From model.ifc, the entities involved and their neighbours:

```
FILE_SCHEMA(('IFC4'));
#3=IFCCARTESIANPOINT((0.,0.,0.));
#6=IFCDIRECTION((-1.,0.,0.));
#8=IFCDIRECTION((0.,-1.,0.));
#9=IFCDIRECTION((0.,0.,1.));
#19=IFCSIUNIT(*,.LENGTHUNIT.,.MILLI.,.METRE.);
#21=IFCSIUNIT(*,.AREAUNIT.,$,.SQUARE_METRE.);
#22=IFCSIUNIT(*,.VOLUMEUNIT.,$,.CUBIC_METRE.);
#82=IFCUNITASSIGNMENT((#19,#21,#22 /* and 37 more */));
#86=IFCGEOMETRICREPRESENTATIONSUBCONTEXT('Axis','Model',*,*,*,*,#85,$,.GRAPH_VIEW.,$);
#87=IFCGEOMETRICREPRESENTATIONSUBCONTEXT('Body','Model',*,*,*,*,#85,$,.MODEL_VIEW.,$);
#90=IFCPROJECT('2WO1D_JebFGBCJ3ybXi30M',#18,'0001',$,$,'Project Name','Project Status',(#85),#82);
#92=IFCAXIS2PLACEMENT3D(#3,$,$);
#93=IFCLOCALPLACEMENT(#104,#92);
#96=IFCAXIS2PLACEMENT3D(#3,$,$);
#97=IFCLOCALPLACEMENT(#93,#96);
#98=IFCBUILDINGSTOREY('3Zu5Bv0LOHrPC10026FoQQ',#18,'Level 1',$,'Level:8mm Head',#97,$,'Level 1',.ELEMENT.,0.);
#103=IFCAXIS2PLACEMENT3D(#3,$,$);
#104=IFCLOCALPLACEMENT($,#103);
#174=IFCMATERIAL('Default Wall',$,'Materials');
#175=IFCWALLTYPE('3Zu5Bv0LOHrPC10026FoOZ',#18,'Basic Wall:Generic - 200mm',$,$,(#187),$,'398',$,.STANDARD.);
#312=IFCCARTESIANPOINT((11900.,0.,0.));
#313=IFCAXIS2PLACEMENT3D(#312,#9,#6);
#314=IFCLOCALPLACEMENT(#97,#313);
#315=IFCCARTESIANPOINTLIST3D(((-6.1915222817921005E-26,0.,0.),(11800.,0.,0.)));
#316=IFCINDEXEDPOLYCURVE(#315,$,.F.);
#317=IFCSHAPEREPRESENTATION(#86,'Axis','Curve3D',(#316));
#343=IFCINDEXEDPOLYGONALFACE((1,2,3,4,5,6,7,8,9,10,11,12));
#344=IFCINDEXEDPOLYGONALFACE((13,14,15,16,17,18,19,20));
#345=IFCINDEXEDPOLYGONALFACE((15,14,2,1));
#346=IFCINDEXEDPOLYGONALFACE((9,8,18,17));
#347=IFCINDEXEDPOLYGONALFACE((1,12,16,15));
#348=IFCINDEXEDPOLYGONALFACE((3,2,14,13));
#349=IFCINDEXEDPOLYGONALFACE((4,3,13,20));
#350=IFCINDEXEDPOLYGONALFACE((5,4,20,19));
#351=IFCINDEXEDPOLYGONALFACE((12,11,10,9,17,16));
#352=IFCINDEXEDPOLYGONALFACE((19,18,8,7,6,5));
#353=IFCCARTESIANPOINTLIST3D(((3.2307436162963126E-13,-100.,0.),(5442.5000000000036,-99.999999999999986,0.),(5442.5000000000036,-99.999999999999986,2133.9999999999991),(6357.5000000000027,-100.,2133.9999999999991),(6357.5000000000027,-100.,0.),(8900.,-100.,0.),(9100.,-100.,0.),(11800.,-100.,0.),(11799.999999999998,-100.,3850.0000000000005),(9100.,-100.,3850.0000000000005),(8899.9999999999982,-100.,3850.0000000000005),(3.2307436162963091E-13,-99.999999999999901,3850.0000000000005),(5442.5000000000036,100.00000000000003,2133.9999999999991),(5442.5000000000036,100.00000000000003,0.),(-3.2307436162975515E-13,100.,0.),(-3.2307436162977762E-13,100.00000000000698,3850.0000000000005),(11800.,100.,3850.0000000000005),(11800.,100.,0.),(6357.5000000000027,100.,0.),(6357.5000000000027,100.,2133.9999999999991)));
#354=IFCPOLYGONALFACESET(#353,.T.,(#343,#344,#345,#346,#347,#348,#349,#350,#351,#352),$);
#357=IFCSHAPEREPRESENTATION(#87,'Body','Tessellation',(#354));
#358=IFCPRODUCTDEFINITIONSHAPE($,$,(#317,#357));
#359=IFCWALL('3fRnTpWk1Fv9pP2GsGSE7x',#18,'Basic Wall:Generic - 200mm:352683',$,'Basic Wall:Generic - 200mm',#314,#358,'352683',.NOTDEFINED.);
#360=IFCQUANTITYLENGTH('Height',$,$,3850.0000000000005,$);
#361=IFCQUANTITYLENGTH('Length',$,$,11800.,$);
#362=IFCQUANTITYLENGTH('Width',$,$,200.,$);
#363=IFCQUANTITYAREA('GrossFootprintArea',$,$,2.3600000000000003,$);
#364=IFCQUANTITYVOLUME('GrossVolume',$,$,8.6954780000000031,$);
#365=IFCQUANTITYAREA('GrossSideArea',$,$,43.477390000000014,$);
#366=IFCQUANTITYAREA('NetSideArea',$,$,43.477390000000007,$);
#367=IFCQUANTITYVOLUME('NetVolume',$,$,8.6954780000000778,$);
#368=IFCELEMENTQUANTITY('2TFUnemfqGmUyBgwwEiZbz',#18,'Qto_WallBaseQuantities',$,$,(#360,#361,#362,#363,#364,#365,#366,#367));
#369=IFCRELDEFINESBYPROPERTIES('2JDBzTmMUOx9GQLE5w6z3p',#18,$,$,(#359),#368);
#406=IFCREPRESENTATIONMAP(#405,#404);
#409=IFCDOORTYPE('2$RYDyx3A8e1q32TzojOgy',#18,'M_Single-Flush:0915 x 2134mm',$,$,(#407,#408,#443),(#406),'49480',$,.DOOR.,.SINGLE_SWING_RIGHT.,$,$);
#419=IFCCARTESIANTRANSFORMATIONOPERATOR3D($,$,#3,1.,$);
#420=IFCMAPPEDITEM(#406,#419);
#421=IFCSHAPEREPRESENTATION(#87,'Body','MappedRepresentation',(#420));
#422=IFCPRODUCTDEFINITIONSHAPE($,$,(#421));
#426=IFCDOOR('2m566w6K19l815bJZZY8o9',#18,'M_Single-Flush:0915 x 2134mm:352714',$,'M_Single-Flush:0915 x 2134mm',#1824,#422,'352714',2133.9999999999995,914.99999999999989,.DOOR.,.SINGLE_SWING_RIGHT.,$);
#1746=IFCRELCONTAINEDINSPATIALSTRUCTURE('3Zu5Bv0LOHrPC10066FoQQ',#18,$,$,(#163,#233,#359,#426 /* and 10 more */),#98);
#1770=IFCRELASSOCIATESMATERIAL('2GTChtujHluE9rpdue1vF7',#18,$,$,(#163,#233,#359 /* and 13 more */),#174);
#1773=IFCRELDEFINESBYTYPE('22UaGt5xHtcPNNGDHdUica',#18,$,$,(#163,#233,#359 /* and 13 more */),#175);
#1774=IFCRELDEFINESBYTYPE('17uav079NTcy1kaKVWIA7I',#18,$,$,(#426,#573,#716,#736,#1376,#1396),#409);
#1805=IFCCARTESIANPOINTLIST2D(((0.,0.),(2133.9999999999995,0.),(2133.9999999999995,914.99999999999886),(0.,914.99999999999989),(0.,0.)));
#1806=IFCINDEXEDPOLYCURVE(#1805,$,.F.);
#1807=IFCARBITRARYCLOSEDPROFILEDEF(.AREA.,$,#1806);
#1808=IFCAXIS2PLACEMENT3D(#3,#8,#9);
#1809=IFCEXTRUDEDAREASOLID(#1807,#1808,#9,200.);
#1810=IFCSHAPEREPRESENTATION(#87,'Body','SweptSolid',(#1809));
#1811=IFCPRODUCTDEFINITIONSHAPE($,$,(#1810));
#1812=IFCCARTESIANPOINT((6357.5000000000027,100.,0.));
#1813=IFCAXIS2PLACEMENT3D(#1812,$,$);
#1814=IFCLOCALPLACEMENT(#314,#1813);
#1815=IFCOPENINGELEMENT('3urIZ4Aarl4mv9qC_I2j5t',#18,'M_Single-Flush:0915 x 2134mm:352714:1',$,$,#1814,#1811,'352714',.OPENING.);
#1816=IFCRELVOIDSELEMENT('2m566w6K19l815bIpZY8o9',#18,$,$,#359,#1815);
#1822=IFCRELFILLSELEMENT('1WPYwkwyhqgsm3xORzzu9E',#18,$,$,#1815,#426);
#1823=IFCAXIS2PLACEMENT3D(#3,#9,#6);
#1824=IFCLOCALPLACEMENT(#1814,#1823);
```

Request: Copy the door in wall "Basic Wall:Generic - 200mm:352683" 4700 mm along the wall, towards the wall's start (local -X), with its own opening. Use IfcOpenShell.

```python
import ifcopenshell
import ifcopenshell.api.feature
import ifcopenshell.api.geometry
import ifcopenshell.api.pset
import ifcopenshell.api.root
import ifcopenshell.geom
import ifcopenshell.util.element
import ifcopenshell.util.placement
import ifcopenshell.util.shape
import ifcopenshell.util.unit

model = ifcopenshell.open("model.ifc")
area_scale = ifcopenshell.util.unit.calculate_unit_scale(model, "AREAUNIT")
volume_scale = ifcopenshell.util.unit.calculate_unit_scale(model, "VOLUMEUNIT")
settings = ifcopenshell.geom.settings()


def volume(element):
    """Net volume in cubic metres, openings subtracted."""
    shape = ifcopenshell.geom.create_shape(settings, element)
    return ifcopenshell.util.shape.get_volume(shape.geometry)


def reuse_history(source, copy):
    """copy_class also copies each property set's owner history, people and application; keep the originals."""
    for rel in copy.IsDefinedBy:
        if rel.is_a("IfcRelDefinesByProperties") and (history := rel.RelatingPropertyDefinition.OwnerHistory):
            rel.RelatingPropertyDefinition.OwnerHistory = source.OwnerHistory
            ifcopenshell.util.element.remove_deep2(model, history)


door = model.by_guid("2m566w6K19l815bJZZY8o9")
opening = door.FillsVoids[0].RelatingOpeningElement
wall = opening.VoidsElements[0].RelatingBuildingElement
before = volume(wall)
shift = ifcopenshell.util.placement.get_local_placement(wall.ObjectPlacement)[:3, 0] * -4700.0

# copy_class copies the void relationship, type, container and properties, but no geometry.
new_opening = ifcopenshell.api.root.copy_class(model, product=opening)
new_opening.Representation = ifcopenshell.util.element.copy_deep(
    model, opening.Representation, exclude=["IfcGeometricRepresentationContext", "IfcRepresentationMap"]
)
new_opening.Name = "M_Single-Flush:0915 x 2134mm"
new_opening.Tag = None
reuse_history(opening, new_opening)
new_door = ifcopenshell.api.root.copy_class(model, product=door)
new_door.Representation = ifcopenshell.util.element.copy_deep(
    model, door.Representation, exclude=["IfcGeometricRepresentationContext", "IfcRepresentationMap"]
)
new_door.Name = "M_Single-Flush:0915 x 2134mm"
new_door.Tag = None
reuse_history(door, new_door)
ifcopenshell.api.feature.add_filling(model, opening=new_opening, element=new_door)

for old, new in ((opening, new_opening), (door, new_door)):
    matrix = ifcopenshell.util.placement.get_local_placement(old.ObjectPlacement)
    matrix[:3, 3] += shift
    ifcopenshell.api.geometry.edit_object_placement(model, product=new, matrix=matrix, is_si=False)

after = volume(wall)
thickness = 0.2  # wall thickness in metres

# Update the wall's stored quantities.
qto = model.by_id(ifcopenshell.util.element.get_pset(wall, "Qto_WallBaseQuantities", should_inherit=False)["id"])
ifcopenshell.api.pset.edit_qto(model, qto=qto, properties={
    "NetSideArea": after / thickness / area_scale,
    "NetVolume": after / volume_scale,
})

print(f"wall volume {before:.3f} -> {after:.3f} m3")

model.write("model-out.ifc")
```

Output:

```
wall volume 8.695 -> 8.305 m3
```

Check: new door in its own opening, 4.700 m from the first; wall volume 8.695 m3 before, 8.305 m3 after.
